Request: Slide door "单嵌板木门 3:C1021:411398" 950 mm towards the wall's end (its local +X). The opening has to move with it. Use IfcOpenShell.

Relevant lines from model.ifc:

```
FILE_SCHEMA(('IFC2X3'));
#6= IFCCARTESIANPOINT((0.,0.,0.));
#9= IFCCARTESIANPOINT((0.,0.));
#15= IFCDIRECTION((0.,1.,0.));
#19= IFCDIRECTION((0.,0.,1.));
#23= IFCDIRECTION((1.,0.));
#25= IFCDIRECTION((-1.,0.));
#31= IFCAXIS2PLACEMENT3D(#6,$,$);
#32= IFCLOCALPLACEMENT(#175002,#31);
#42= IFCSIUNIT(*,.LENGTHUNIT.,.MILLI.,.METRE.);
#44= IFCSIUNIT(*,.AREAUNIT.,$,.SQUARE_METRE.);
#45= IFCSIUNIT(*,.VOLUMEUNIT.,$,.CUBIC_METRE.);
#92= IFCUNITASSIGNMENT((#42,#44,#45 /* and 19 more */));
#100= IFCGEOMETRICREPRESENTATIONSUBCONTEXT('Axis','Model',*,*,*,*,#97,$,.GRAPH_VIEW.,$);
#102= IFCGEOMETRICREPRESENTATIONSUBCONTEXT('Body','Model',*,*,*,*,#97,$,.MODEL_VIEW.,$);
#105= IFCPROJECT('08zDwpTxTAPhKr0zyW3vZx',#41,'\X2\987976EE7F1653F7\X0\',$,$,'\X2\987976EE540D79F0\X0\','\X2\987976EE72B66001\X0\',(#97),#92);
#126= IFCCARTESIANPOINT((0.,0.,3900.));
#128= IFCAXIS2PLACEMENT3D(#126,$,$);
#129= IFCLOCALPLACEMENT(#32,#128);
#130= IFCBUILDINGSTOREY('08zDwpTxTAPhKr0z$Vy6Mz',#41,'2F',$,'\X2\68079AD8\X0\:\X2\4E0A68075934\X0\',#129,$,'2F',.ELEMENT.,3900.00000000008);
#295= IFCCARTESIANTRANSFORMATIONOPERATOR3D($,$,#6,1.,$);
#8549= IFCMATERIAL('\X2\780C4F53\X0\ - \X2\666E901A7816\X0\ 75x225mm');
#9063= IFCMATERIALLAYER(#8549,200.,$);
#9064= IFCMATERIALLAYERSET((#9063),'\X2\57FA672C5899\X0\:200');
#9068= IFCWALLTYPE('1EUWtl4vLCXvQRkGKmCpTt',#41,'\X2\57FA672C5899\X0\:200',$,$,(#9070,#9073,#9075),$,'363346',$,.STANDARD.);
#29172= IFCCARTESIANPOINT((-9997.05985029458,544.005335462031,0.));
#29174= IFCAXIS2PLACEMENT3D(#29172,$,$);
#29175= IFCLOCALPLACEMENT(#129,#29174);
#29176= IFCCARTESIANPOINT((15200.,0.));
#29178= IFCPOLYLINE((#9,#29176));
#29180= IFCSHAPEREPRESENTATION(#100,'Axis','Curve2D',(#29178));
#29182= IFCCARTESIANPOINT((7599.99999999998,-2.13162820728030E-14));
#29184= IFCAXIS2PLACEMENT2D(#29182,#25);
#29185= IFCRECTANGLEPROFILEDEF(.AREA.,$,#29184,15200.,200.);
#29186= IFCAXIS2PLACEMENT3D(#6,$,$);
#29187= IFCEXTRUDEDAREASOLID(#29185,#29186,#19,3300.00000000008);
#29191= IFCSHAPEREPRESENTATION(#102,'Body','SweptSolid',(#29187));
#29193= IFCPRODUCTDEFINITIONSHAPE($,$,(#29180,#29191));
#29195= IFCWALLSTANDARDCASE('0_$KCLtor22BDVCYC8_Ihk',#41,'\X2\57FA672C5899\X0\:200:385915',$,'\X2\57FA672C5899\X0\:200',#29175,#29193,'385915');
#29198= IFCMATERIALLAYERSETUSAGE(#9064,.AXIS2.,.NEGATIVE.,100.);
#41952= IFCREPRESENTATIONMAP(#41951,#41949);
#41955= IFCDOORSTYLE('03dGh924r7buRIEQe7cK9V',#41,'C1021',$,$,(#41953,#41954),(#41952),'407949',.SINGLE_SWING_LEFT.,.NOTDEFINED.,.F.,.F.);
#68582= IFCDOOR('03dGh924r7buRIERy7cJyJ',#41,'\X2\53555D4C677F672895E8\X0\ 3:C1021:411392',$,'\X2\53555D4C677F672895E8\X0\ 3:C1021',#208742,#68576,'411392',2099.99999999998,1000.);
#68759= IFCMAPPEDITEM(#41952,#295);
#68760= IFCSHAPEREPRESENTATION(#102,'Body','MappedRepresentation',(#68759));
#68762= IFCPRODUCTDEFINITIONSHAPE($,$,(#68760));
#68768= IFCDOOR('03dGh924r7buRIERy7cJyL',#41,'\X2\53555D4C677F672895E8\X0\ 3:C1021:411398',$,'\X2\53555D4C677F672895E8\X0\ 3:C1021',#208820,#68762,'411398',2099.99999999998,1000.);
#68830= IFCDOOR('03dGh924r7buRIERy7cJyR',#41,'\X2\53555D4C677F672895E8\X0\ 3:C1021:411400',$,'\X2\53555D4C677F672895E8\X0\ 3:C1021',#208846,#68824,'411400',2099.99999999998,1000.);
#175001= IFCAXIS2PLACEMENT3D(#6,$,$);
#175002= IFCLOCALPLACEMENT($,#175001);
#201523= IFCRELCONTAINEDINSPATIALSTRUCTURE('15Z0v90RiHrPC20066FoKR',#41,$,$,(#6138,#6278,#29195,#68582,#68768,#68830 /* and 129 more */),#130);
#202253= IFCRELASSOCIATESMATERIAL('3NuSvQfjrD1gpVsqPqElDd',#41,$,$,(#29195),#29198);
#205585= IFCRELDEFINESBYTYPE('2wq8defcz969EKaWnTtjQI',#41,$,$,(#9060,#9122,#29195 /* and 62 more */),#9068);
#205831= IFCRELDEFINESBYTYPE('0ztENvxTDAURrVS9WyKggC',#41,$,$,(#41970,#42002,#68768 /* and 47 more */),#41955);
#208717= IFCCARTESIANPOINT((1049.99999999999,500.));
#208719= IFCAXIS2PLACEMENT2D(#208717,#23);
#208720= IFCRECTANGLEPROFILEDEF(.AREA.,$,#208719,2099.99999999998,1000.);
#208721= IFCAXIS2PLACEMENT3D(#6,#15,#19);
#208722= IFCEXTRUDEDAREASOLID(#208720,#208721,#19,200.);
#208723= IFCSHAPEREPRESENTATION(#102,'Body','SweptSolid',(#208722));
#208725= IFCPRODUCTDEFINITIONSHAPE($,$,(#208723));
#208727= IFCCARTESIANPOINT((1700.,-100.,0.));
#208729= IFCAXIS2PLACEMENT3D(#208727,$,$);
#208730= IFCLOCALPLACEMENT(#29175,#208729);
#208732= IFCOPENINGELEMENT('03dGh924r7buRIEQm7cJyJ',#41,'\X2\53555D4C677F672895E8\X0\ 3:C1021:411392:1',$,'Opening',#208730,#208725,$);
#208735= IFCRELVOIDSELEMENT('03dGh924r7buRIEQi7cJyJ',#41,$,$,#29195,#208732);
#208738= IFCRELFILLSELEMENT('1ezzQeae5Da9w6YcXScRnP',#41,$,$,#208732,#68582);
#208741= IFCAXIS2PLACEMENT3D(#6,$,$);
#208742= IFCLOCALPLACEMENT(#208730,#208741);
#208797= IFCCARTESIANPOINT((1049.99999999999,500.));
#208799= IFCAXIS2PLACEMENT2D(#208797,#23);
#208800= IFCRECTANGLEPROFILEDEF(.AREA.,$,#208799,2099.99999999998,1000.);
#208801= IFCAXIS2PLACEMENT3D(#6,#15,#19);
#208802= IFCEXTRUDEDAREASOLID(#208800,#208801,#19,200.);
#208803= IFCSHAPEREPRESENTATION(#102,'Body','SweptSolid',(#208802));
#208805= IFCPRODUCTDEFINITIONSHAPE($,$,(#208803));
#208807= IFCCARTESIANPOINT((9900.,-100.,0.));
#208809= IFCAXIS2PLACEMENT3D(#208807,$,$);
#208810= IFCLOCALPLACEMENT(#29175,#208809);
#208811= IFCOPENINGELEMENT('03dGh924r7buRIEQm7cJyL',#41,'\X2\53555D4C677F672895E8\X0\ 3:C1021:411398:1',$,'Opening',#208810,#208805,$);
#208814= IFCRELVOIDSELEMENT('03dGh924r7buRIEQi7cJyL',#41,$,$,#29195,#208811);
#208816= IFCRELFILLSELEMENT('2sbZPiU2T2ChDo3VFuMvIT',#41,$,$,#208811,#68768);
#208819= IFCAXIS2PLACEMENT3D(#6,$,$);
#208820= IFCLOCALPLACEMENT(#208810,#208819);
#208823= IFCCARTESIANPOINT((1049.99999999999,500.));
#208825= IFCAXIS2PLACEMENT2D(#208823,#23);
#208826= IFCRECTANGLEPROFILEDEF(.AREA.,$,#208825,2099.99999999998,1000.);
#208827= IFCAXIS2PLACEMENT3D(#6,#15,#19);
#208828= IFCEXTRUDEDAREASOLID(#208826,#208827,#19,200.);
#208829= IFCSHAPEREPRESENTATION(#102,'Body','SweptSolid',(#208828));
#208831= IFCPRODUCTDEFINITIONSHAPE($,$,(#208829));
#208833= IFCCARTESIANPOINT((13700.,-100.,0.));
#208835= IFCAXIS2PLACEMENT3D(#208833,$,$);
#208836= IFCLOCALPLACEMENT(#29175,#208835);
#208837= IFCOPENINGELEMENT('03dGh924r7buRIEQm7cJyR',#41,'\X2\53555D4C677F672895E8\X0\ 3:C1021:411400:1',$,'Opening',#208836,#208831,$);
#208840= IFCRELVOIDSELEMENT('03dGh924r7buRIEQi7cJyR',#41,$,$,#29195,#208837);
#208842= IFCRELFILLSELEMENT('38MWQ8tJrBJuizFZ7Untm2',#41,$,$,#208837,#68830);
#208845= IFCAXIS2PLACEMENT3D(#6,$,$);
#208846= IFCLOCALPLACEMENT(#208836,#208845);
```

```python
import ifcopenshell
import ifcopenshell.api.geometry
import ifcopenshell.util.placement
import ifcopenshell.util.unit

model = ifcopenshell.open("model.ifc")
unit_scale = ifcopenshell.util.unit.calculate_unit_scale(model)

door = model.by_id(68768)
opening = door.FillsVoids[0].RelatingOpeningElement
wall = opening.VoidsElements[0].RelatingBuildingElement

wall_matrix = ifcopenshell.util.placement.get_local_placement(wall.ObjectPlacement)
shift = wall_matrix[:3, 0] * 0.95 / unit_scale
before = ifcopenshell.util.placement.get_local_placement(door.ObjectPlacement)[:3, 3].copy()

# The door is placed relative to its opening, so it follows when the opening moves.
matrix = ifcopenshell.util.placement.get_local_placement(opening.ObjectPlacement)
matrix[:3, 3] += shift
ifcopenshell.api.geometry.edit_object_placement(
    model, product=opening, matrix=matrix, is_si=False, should_transform_children=True
)

after = ifcopenshell.util.placement.get_local_placement(door.ObjectPlacement)[:3, 3]
print("door moved by", (after - before).round(3) + 0.0)

model.write("model_updated.ifc")
```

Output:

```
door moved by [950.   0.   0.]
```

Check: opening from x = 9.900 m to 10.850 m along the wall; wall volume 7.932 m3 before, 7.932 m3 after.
